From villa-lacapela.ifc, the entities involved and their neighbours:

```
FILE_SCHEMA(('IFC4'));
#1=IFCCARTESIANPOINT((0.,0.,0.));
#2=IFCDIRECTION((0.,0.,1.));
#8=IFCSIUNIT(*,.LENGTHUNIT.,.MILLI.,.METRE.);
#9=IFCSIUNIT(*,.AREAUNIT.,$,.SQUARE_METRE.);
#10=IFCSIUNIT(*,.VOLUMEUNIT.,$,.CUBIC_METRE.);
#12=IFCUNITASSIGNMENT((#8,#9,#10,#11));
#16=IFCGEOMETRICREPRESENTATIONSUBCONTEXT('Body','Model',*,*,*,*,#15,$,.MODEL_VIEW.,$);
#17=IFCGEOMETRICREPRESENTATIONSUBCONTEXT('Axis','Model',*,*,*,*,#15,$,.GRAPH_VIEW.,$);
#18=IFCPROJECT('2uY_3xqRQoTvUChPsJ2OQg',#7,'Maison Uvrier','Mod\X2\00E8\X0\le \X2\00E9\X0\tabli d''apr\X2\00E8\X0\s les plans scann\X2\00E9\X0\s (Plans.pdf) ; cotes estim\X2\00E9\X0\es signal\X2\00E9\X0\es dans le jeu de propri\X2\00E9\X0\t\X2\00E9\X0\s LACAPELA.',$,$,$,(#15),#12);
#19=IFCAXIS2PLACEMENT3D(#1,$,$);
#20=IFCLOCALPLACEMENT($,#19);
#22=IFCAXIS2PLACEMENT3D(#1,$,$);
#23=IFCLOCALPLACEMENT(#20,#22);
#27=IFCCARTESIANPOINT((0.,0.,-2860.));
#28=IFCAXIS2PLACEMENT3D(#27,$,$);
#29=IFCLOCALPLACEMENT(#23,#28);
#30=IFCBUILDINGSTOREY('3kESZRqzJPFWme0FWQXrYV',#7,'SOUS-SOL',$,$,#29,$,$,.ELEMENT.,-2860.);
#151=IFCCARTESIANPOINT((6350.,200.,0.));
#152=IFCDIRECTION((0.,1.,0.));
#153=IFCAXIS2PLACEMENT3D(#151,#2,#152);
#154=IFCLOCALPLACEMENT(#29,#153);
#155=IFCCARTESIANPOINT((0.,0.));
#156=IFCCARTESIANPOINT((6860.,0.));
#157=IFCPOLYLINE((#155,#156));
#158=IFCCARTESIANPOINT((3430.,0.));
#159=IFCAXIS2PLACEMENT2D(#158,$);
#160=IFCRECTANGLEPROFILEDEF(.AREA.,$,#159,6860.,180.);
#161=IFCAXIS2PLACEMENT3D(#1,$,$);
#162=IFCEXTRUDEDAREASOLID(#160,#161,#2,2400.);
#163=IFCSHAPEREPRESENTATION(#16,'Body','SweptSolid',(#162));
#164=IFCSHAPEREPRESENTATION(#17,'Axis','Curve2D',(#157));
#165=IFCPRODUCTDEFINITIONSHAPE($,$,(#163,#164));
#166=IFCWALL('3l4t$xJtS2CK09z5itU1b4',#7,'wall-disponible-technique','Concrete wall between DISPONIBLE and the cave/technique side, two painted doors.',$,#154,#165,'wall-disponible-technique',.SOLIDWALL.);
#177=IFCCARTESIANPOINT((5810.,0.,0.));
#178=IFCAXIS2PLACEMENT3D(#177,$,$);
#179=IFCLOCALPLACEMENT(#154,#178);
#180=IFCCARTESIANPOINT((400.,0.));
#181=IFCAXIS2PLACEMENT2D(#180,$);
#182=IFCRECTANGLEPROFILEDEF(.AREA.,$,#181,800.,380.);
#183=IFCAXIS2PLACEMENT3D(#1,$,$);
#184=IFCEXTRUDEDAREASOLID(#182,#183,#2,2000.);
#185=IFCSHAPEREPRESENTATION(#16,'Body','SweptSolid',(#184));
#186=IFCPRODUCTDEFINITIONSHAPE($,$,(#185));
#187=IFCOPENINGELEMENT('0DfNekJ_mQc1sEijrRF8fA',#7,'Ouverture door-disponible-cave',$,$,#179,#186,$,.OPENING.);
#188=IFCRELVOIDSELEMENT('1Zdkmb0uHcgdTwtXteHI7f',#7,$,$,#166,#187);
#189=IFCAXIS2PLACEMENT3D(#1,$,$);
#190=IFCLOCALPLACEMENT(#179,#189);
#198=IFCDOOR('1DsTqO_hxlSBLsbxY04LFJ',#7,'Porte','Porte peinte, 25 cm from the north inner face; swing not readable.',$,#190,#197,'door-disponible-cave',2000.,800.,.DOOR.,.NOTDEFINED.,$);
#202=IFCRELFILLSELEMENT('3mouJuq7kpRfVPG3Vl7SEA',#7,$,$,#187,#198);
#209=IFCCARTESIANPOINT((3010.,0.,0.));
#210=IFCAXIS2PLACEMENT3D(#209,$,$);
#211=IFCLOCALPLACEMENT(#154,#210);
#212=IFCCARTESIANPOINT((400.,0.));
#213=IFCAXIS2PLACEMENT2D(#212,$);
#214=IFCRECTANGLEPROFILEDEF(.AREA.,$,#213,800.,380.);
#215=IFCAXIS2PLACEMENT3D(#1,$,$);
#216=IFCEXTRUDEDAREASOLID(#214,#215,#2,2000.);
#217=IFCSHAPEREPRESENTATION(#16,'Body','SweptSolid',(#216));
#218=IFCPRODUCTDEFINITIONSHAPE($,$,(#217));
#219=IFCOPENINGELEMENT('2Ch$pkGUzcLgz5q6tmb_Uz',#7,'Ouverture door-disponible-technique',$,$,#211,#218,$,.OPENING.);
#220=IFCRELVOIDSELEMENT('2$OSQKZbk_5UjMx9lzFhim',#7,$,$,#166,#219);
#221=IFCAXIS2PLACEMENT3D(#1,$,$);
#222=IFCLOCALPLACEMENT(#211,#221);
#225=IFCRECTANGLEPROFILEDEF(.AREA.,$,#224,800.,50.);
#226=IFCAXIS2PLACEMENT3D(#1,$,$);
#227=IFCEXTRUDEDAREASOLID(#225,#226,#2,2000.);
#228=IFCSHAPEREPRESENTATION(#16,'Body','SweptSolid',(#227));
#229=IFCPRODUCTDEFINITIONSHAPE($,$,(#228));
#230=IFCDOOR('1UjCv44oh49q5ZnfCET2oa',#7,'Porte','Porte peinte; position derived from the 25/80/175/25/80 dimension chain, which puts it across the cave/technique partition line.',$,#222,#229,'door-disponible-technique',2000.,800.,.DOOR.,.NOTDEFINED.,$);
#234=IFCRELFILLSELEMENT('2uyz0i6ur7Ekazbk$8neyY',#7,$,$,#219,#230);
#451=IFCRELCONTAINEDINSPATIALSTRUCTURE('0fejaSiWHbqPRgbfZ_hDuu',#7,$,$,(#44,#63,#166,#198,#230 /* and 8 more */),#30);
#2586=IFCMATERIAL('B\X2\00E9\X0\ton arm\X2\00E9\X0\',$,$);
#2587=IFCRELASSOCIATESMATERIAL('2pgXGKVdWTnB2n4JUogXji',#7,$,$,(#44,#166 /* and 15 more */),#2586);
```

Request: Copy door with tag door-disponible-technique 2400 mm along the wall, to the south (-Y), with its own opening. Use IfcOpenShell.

```python
import ifcopenshell
import ifcopenshell.api.feature
import ifcopenshell.api.geometry
import ifcopenshell.api.root
import ifcopenshell.geom
import ifcopenshell.util.element
import ifcopenshell.util.placement
import ifcopenshell.util.shape

model = ifcopenshell.open("villa-lacapela.ifc")
settings = ifcopenshell.geom.settings()


def volume(element):
    """Net volume in cubic metres, openings subtracted."""
    shape = ifcopenshell.geom.create_shape(settings, element)
    return ifcopenshell.util.shape.get_volume(shape.geometry)


def reuse_history(source, copy):
    """copy_class also copies each property set's owner history, people and application; keep the originals."""
    for rel in copy.IsDefinedBy:
        if rel.is_a("IfcRelDefinesByProperties") and (history := rel.RelatingPropertyDefinition.OwnerHistory):
            rel.RelatingPropertyDefinition.OwnerHistory = source.OwnerHistory
            ifcopenshell.util.element.remove_deep2(model, history)


door = model.by_guid("1UjCv44oh49q5ZnfCET2oa")
opening = door.FillsVoids[0].RelatingOpeningElement
wall = opening.VoidsElements[0].RelatingBuildingElement
before = volume(wall)
shift = ifcopenshell.util.placement.get_local_placement(wall.ObjectPlacement)[:3, 0] * -2400.0

# copy_class copies the void relationship, type, container and properties, but no geometry.
new_opening = ifcopenshell.api.root.copy_class(model, product=opening)
new_opening.Representation = ifcopenshell.util.element.copy_deep(
    model, opening.Representation, exclude=["IfcGeometricRepresentationContext", "IfcRepresentationMap"]
)
new_door = ifcopenshell.api.root.copy_class(model, product=door)
new_door.Representation = ifcopenshell.util.element.copy_deep(
    model, door.Representation, exclude=["IfcGeometricRepresentationContext", "IfcRepresentationMap"]
)
new_door.Tag = None
reuse_history(door, new_door)
ifcopenshell.api.feature.add_filling(model, opening=new_opening, element=new_door)

for old, new in ((opening, new_opening), (door, new_door)):
    matrix = ifcopenshell.util.placement.get_local_placement(old.ObjectPlacement)
    matrix[:3, 3] += shift
    ifcopenshell.api.geometry.edit_object_placement(model, product=new, matrix=matrix, is_si=False)

after = volume(wall)

print(f"wall volume {before:.3f} -> {after:.3f} m3")

model.write("villa-lacapela_edited.ifc")
```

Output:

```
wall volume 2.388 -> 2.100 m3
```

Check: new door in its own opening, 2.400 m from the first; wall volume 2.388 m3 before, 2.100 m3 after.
